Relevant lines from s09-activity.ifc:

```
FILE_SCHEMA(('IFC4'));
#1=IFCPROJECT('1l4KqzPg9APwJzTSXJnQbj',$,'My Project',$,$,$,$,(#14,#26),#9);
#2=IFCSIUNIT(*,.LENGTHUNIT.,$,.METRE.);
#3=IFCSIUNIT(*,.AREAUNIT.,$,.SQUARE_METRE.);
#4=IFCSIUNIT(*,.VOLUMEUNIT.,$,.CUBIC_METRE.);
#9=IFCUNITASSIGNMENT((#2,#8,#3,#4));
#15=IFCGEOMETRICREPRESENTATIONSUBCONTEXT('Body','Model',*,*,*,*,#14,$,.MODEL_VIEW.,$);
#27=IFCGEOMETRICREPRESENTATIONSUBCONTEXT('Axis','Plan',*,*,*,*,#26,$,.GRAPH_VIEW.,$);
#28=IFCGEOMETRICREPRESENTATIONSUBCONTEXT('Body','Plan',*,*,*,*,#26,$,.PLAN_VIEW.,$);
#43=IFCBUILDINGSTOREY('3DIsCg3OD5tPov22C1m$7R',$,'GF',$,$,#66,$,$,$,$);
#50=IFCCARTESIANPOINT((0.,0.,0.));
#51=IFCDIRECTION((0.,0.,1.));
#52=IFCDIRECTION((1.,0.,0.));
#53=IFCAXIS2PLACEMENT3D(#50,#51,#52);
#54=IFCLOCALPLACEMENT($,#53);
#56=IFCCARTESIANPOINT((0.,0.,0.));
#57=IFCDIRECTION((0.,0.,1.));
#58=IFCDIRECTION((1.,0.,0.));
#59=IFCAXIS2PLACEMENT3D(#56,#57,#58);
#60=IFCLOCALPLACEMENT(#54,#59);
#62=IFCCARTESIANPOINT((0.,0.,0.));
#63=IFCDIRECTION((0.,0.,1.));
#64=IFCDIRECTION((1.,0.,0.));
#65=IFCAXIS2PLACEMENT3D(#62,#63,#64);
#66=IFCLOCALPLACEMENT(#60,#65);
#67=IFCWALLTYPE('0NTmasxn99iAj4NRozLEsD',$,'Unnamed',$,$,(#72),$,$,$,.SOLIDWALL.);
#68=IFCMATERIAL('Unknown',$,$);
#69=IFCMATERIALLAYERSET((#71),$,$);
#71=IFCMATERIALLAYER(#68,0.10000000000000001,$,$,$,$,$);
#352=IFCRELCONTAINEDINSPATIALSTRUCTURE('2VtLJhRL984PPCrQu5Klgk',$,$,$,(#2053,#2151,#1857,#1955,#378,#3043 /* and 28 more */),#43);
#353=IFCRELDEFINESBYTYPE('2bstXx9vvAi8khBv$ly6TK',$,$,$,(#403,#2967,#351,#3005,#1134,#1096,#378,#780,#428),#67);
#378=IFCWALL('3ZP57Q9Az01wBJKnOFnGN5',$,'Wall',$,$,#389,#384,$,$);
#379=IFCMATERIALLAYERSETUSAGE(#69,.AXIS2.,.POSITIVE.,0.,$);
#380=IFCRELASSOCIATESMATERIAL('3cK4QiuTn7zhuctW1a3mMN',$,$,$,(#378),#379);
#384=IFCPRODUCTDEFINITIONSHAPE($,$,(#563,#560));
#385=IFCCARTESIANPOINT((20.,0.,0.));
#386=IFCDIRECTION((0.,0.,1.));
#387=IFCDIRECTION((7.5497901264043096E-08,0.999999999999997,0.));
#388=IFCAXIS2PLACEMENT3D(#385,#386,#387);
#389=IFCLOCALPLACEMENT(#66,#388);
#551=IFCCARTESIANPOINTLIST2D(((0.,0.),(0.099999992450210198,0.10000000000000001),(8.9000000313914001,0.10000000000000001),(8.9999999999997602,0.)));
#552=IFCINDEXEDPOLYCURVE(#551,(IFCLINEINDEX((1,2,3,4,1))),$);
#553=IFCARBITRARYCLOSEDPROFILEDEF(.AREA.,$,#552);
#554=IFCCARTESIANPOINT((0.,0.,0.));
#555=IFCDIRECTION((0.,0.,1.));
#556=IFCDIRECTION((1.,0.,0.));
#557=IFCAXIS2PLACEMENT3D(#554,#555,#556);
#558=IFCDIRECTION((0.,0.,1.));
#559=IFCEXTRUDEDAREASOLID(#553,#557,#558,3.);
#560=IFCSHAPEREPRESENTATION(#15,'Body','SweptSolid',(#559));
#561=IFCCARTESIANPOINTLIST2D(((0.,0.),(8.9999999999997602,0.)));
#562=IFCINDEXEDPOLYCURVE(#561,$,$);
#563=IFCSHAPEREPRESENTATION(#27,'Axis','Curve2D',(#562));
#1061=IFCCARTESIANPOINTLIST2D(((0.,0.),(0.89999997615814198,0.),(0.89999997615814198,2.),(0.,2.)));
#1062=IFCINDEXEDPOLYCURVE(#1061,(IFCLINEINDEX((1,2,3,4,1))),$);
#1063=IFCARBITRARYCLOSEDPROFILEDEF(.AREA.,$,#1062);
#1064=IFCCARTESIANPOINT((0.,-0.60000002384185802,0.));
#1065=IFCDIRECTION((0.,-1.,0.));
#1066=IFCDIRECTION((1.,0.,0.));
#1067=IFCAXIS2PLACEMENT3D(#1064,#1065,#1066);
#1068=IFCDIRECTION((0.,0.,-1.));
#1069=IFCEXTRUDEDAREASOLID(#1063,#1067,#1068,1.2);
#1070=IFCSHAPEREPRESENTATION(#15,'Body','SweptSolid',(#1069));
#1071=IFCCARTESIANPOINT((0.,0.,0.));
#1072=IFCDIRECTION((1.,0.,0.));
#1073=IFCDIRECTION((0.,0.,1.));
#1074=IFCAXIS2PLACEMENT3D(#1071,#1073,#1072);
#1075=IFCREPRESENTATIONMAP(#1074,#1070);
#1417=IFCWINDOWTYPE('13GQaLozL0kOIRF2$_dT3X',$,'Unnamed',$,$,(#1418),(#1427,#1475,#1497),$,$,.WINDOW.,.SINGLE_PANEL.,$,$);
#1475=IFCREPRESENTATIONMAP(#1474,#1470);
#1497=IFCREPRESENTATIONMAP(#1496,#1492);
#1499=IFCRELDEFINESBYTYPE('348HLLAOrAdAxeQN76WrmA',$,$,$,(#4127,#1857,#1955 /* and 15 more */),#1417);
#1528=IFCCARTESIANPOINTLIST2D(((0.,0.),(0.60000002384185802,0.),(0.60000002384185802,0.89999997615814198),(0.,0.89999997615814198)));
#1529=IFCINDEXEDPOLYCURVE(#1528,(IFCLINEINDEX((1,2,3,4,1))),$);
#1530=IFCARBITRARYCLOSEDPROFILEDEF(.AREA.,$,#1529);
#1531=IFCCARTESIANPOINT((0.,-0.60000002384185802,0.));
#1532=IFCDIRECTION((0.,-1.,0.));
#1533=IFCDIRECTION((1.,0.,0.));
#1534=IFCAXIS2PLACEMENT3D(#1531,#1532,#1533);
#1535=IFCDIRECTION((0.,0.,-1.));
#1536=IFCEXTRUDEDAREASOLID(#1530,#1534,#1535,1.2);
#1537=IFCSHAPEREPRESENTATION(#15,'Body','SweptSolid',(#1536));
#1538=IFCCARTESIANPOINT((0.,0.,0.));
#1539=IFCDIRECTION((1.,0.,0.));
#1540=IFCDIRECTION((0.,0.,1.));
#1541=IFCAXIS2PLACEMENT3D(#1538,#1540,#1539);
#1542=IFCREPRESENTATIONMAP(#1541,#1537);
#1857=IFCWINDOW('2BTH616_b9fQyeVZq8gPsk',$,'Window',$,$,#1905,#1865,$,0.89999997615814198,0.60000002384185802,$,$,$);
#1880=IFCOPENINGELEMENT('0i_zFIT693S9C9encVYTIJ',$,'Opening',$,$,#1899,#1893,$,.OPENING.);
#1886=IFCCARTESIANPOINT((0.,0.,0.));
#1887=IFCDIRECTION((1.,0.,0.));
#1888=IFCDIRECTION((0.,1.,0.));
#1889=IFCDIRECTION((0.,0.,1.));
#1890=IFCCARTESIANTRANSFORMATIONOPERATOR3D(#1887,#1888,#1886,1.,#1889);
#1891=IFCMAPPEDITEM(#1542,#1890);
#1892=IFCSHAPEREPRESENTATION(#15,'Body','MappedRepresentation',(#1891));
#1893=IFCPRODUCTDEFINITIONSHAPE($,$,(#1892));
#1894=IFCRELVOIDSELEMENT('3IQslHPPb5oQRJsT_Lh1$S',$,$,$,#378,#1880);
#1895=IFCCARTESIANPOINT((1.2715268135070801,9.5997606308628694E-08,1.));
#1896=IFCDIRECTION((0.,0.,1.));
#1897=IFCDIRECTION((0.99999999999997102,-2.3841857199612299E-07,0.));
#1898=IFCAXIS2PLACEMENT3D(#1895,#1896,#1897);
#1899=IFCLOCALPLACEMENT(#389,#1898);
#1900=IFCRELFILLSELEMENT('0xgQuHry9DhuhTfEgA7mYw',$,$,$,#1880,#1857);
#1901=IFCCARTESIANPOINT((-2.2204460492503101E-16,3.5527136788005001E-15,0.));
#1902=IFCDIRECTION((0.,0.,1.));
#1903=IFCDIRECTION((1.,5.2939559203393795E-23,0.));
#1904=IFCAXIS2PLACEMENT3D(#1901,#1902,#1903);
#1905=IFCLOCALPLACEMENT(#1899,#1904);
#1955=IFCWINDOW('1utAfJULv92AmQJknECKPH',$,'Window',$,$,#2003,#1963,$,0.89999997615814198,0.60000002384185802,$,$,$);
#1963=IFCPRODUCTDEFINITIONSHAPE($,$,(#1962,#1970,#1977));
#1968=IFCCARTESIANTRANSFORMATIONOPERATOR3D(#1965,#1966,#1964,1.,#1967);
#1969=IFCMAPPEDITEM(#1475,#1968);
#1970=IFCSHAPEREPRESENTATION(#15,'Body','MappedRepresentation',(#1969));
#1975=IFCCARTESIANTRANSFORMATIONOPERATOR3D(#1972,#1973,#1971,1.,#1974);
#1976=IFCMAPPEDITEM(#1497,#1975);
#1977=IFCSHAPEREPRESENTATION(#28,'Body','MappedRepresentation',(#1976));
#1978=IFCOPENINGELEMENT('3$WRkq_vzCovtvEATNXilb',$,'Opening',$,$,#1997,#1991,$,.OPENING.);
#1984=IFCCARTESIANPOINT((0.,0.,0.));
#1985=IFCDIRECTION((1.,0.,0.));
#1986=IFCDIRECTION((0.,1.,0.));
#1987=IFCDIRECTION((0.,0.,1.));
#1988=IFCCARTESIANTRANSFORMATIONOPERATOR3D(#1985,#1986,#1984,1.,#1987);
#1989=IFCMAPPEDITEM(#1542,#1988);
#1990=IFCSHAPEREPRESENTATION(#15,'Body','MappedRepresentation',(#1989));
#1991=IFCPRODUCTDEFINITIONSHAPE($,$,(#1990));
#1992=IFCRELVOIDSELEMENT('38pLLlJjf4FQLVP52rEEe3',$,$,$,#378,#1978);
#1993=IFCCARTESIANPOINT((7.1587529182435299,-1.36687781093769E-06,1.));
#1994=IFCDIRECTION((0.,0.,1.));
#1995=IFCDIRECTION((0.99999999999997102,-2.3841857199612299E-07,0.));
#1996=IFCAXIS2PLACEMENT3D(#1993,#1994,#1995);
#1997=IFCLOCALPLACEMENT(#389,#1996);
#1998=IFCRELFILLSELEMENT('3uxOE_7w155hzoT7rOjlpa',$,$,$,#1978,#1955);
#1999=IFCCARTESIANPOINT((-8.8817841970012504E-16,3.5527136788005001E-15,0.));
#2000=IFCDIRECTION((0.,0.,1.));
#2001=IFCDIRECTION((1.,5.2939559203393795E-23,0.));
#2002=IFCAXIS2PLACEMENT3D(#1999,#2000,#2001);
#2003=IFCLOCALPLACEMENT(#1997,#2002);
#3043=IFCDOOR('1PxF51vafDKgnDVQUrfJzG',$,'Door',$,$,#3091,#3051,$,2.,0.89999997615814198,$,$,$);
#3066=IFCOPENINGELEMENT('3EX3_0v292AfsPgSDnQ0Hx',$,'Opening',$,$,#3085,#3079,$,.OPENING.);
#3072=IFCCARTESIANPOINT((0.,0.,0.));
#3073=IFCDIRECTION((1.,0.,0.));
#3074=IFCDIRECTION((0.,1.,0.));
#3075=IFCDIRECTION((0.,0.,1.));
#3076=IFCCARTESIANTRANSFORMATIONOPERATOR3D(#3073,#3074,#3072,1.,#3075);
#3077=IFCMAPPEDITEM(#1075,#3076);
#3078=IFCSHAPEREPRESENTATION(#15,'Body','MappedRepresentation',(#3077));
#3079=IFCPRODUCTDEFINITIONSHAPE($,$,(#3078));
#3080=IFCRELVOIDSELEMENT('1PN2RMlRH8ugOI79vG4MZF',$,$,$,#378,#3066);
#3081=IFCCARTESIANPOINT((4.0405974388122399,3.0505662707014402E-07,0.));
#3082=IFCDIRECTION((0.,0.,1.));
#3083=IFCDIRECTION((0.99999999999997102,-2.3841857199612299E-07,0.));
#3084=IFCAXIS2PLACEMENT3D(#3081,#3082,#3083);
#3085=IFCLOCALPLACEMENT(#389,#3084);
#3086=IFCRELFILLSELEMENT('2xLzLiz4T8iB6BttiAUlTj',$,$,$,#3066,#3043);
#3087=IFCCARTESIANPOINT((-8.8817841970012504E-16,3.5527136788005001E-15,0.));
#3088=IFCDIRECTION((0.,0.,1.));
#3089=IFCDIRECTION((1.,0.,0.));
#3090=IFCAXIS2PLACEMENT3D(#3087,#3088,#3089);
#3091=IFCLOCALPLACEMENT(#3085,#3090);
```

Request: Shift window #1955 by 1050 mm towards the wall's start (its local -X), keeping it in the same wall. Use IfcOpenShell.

```python
import ifcopenshell
import ifcopenshell.api.geometry
import ifcopenshell.util.placement

model = ifcopenshell.open("s09-activity.ifc")

window = model.by_guid("1utAfJULv92AmQJknECKPH")
opening = window.FillsVoids[0].RelatingOpeningElement
wall = opening.VoidsElements[0].RelatingBuildingElement

wall_matrix = ifcopenshell.util.placement.get_local_placement(wall.ObjectPlacement)
shift = wall_matrix[:3, 0] * -1.05
before = ifcopenshell.util.placement.get_local_placement(window.ObjectPlacement)[:3, 3].copy()

# The window is placed relative to its opening, so it follows when the opening moves.
matrix = ifcopenshell.util.placement.get_local_placement(opening.ObjectPlacement)
matrix[:3, 3] += shift
ifcopenshell.api.geometry.edit_object_placement(
    model, product=opening, matrix=matrix, is_si=False, should_transform_children=True
)

after = ifcopenshell.util.placement.get_local_placement(window.ObjectPlacement)[:3, 3]
print("window moved by", (after - before).round(3) + 0.0)

model.write("s09-activity-out.ifc")
```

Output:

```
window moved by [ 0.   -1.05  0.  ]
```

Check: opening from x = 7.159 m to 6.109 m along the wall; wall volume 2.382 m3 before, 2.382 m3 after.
